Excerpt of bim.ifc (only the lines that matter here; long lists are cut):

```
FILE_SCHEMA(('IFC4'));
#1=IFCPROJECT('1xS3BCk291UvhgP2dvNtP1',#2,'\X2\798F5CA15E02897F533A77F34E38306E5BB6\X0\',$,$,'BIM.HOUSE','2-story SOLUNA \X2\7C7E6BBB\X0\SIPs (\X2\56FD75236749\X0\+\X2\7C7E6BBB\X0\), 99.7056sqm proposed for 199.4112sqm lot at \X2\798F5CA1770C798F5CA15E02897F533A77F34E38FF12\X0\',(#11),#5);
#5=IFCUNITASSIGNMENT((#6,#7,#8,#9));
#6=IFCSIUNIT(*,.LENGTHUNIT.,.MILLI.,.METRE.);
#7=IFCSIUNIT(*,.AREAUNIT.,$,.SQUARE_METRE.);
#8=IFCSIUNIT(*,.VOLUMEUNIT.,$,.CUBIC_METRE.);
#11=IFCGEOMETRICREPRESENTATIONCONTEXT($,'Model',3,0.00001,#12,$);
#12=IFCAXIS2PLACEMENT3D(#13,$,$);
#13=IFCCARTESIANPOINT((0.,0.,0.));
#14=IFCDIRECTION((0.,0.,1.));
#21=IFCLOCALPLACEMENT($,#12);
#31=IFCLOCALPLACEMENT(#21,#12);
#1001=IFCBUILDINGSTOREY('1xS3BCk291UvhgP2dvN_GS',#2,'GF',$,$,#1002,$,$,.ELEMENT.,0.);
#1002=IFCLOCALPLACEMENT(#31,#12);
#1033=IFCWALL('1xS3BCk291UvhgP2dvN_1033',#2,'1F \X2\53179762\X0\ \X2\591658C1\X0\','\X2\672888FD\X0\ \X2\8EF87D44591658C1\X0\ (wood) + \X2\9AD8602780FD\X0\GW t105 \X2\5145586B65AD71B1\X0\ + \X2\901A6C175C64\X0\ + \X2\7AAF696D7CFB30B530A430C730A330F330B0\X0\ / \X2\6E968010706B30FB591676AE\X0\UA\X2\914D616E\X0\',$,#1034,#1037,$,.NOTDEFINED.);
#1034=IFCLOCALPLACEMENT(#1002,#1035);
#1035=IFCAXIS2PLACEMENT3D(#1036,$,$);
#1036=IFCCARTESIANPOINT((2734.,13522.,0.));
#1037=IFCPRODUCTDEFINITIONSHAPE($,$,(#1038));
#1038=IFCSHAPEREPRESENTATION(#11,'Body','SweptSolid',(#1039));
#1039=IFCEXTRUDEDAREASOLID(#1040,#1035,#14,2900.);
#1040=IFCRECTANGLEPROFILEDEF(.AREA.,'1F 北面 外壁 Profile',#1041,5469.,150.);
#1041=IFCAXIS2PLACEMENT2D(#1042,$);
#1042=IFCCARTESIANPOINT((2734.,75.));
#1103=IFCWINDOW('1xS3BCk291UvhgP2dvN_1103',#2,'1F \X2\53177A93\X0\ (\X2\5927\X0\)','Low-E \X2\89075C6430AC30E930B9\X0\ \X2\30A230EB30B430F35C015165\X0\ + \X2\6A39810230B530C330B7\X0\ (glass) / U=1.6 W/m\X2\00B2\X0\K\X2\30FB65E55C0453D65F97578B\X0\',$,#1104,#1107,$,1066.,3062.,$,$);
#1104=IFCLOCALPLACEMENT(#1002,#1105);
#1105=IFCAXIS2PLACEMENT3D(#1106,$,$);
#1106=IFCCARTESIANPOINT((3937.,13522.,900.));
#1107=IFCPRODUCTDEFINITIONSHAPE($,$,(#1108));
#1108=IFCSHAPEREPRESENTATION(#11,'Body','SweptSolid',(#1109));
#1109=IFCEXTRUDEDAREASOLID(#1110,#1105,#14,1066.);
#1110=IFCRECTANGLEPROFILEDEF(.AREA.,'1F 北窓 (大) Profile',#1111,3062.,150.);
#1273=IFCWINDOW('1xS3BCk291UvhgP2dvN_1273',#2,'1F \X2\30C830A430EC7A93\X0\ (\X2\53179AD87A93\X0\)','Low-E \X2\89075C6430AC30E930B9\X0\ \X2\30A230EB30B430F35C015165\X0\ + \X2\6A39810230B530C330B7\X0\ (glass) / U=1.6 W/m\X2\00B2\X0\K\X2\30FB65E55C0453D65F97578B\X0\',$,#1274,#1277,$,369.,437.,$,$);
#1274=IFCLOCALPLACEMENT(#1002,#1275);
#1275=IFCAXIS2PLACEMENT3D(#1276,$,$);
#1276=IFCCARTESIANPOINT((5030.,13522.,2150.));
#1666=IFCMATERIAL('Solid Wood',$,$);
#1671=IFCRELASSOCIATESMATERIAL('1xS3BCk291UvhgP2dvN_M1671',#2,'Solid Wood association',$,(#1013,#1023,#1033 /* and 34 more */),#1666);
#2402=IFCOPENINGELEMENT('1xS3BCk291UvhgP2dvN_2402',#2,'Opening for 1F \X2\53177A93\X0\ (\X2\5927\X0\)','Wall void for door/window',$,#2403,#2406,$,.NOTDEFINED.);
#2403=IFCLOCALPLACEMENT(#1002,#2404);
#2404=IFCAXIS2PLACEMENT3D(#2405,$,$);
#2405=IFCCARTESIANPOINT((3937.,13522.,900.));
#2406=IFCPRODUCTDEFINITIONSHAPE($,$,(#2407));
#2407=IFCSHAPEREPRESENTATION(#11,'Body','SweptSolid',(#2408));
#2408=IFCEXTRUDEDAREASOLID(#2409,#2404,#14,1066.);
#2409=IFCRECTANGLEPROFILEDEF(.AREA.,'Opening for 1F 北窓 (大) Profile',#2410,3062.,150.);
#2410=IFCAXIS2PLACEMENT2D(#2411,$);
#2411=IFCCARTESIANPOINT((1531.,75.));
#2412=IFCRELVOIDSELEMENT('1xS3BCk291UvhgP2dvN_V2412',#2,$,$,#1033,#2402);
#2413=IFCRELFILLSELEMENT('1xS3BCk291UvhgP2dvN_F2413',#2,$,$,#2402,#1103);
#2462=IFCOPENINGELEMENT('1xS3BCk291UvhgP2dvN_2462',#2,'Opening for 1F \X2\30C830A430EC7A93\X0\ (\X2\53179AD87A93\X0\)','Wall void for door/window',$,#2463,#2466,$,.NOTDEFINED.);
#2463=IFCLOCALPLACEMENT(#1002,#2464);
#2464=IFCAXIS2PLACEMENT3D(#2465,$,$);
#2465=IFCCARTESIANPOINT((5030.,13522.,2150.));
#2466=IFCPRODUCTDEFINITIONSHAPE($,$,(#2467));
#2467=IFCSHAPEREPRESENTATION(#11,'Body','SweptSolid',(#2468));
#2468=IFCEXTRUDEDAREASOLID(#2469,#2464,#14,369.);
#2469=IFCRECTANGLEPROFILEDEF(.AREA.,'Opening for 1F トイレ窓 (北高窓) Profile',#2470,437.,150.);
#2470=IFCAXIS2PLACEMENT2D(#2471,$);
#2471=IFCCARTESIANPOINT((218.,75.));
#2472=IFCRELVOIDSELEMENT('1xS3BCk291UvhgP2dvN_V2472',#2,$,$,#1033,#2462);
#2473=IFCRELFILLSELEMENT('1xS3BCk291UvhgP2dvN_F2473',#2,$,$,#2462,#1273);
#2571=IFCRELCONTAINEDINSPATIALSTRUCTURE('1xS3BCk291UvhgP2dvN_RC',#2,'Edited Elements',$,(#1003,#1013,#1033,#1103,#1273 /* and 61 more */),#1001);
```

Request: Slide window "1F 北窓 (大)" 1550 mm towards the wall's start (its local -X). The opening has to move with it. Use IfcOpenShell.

```python
import ifcopenshell
import ifcopenshell.api.geometry
import ifcopenshell.util.placement

model = ifcopenshell.open("bim.ifc")

window = model.by_guid("1xS3BCk291UvhgP2dvN_1103")
opening = window.FillsVoids[0].RelatingOpeningElement
wall = opening.VoidsElements[0].RelatingBuildingElement

wall_matrix = ifcopenshell.util.placement.get_local_placement(wall.ObjectPlacement)
shift = wall_matrix[:3, 0] * -1550.0
before = ifcopenshell.util.placement.get_local_placement(window.ObjectPlacement)[:3, 3].copy()

# The window is not placed relative to its opening, so move both.
for product in (opening, window):
    matrix = ifcopenshell.util.placement.get_local_placement(product.ObjectPlacement)
    matrix[:3, 3] += shift
    ifcopenshell.api.geometry.edit_object_placement(model, product=product, matrix=matrix, is_si=False)

after = ifcopenshell.util.placement.get_local_placement(window.ObjectPlacement)[:3, 3]
print("window moved by", (after - before).round(3) + 0.0)

model.write("bim_edited.ifc")
```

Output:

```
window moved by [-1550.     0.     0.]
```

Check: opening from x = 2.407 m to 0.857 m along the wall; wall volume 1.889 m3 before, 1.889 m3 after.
